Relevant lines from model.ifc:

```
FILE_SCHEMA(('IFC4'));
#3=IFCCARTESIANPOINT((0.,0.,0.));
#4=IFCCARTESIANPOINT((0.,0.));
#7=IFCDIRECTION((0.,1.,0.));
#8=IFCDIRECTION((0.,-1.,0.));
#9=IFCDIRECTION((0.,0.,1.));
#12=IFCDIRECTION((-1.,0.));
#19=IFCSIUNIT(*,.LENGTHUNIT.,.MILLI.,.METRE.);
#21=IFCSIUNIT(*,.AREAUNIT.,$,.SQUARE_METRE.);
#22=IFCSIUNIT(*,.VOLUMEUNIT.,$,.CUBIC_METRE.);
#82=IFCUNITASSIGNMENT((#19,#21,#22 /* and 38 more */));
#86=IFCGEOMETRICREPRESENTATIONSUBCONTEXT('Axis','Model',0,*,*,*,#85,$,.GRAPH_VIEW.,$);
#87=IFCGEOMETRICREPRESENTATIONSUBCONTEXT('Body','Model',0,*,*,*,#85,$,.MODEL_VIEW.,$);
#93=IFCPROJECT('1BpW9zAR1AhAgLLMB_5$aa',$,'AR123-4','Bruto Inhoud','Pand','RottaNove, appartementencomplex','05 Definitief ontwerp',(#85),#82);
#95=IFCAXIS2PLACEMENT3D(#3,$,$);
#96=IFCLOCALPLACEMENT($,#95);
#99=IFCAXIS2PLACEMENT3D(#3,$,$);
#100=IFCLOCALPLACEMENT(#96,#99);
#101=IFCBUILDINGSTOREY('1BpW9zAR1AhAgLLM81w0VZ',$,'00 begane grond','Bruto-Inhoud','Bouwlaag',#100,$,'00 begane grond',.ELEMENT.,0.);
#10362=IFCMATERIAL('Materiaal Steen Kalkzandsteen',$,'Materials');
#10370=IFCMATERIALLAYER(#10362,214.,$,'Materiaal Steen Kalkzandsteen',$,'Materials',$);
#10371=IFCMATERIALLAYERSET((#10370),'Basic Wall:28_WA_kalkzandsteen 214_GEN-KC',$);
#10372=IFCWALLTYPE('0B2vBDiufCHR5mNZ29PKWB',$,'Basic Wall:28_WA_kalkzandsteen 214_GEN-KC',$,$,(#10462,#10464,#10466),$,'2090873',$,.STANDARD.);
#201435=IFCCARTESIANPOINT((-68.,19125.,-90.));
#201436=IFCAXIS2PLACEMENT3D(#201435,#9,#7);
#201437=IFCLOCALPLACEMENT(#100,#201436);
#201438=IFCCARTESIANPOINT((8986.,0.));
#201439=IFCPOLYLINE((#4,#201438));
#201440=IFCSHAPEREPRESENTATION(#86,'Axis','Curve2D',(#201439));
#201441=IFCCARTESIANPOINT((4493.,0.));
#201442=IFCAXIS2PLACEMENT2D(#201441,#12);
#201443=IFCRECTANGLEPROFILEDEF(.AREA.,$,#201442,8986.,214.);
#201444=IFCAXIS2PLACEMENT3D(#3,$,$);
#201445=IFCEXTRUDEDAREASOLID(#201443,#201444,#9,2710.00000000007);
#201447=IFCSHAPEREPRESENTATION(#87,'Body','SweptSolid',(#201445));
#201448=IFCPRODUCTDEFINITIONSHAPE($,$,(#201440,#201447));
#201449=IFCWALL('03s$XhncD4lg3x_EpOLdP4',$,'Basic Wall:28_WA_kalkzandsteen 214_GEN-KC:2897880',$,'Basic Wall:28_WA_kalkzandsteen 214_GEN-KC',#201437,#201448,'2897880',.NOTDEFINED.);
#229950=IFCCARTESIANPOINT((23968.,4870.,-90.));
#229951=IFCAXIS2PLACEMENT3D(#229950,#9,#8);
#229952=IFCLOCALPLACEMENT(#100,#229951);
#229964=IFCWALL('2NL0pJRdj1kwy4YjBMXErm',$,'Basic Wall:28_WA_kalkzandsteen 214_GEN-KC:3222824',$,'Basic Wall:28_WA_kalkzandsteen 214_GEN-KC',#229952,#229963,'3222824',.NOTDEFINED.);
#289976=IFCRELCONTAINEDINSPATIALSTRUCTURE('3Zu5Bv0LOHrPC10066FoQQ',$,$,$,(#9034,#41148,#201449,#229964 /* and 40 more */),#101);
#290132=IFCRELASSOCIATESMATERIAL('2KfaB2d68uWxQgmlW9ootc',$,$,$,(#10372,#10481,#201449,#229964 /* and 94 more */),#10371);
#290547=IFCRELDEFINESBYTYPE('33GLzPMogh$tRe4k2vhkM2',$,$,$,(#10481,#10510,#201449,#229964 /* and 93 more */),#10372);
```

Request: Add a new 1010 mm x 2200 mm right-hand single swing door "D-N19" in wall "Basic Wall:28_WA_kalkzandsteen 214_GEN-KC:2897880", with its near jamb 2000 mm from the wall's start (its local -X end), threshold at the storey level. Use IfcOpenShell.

```python
import numpy as np
import ifcopenshell
import ifcopenshell.api.feature
import ifcopenshell.api.geometry
import ifcopenshell.api.root
import ifcopenshell.api.spatial
import ifcopenshell.geom
import ifcopenshell.util.element
import ifcopenshell.util.placement
import ifcopenshell.util.representation
import ifcopenshell.util.shape
import ifcopenshell.util.unit

model = ifcopenshell.open("model.ifc")
unit_scale = ifcopenshell.util.unit.calculate_unit_scale(model)
settings = ifcopenshell.geom.settings()


def volume(element):
    """Net volume in cubic metres, openings subtracted."""
    shape = ifcopenshell.geom.create_shape(settings, element)
    return ifcopenshell.util.shape.get_volume(shape.geometry)


wall = model.by_id(201449)
storey = ifcopenshell.util.element.get_container(wall, ifc_class="IfcBuildingStorey")
context = ifcopenshell.util.representation.get_context(model, "Model", "Body", "MODEL_VIEW")
before = volume(wall)

width, height, from_end, sill = 1.01, 2.2, 2, 0.0  # metres

# The wall runs along its own X axis, and the end named is its -X end.
wall_shape = ifcopenshell.geom.create_shape(settings, wall)
x, y, z = ifcopenshell.util.shape.get_vertices(wall_shape.geometry).T
start = x.min() + from_end
face, thickness = float(y.min()), float(y.max() - y.min())
wall_matrix = ifcopenshell.util.placement.get_local_placement(wall.ObjectPlacement)
level = ifcopenshell.util.placement.get_local_placement(storey.ObjectPlacement)[2, 3]


def in_wall(x, y):
    """Placement at x, y metres in the wall's axes, at sill height."""
    matrix = wall_matrix.copy()
    matrix[:, 3] = wall_matrix @ np.array([x / unit_scale, y / unit_scale, 0.0, 1.0])
    matrix[2, 3] = level + sill / unit_scale
    return matrix


# Opening: a box that overshoots both wall faces by 50 mm.
opening = ifcopenshell.api.root.create_entity(model, ifc_class="IfcOpeningElement", predefined_type="OPENING")
box = ifcopenshell.api.geometry.add_wall_representation(
    model, context=context, length=width, height=height, thickness=thickness + 0.1
)
ifcopenshell.api.geometry.assign_representation(model, product=opening, representation=box)
ifcopenshell.api.geometry.edit_object_placement(model, product=opening, matrix=in_wall(start, face - 0.05), is_si=False)
ifcopenshell.api.feature.add_feature(model, feature=opening, element=wall)

door = ifcopenshell.api.root.create_entity(model, ifc_class="IfcDoor", name="D-N19", predefined_type="DOOR")
door.OverallWidth, door.OverallHeight = width / unit_scale, height / unit_scale
door.OperationType = "SINGLE_SWING_RIGHT"
body = ifcopenshell.api.geometry.add_door_representation(
    model,
    context=context,
    overall_width=door.OverallWidth,
    overall_height=door.OverallHeight,
    operation_type="SINGLE_SWING_RIGHT",
    lining_properties={"LiningDepth": thickness / unit_scale, "ThresholdDepth": thickness / unit_scale},
)
ifcopenshell.api.geometry.assign_representation(model, product=door, representation=body)
ifcopenshell.api.spatial.assign_container(model, products=[door], relating_structure=storey)
ifcopenshell.api.feature.add_filling(model, opening=opening, element=door)

# The lining spans the wall, so the door starts at the wall face.
ifcopenshell.api.geometry.edit_object_placement(model, product=door, matrix=in_wall(start, face), is_si=False)

after = volume(wall)

print(f"wall volume {before:.3f} -> {after:.3f} m3")

model.write("model_edited.ifc")
```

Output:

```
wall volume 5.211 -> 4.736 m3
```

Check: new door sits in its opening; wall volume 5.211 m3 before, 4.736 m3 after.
